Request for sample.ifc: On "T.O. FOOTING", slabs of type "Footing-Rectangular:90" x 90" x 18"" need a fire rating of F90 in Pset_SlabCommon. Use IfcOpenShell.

First a look at what the model holds.

```python
import ifcopenshell
import ifcopenshell.util.element

model = ifcopenshell.open("sample.ifc")
print(model.schema)
storey = next(s for s in model.by_type("IfcBuildingStorey") if s.Name == "T.O. FOOTING")
slabs = [e for e in ifcopenshell.util.element.get_decomposition(storey) if e.is_a("IfcSlab")]
seen = {}
for e in slabs:
    element_type = ifcopenshell.util.element.get_type(e)
    key = (element_type.Name if element_type != e and element_type else None, ifcopenshell.util.element.get_pset(e, "Pset_SlabCommon", "FireRating"))
    seen[key] = seen.get(key, 0) + 1
for (name, value), count in sorted(seen.items(), key=str):
    print(count, "x", name, "|", value)
```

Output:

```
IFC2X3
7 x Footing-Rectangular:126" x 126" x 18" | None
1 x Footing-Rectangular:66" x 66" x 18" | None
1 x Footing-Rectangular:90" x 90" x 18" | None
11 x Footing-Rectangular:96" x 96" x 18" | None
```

```python
import ifcopenshell
import ifcopenshell.api.pset
import ifcopenshell.util.element

model = ifcopenshell.open("sample.ifc")

storey = next(s for s in model.by_type("IfcBuildingStorey") if s.Name == "T.O. FOOTING")
slabs = [e for e in ifcopenshell.util.element.get_decomposition(storey) if e.is_a("IfcSlab")]

count = 0
for e in slabs:
    element_type = ifcopenshell.util.element.get_type(e)
    if element_type in (None, e) or element_type.Name != 'Footing-Rectangular:90" x 90" x 18"':
        continue
    # add_pset returns the element's existing set when there is one.
    pset = ifcopenshell.api.pset.add_pset(model, product=e, name="Pset_SlabCommon")
    ifcopenshell.api.pset.edit_pset(model, pset=pset, properties={"FireRating": "F90"})
    count += 1

print(count, "slabs updated")

model.write("sample_v2.ifc")
```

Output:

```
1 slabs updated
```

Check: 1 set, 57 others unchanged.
